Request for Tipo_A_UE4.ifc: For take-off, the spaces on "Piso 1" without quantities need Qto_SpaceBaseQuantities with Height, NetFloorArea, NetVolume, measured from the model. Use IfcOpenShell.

First a look at what the model holds.

```python
import ifcopenshell
import ifcopenshell.util.element
import ifcopenshell.util.unit

model = ifcopenshell.open("Tipo_A_UE4.ifc")
print(model.schema)
for unit_type in ("LENGTHUNIT", "AREAUNIT", "VOLUMEUNIT"):
    print(unit_type, ifcopenshell.util.unit.calculate_unit_scale(model, unit_type))
storey = next(s for s in model.by_type("IfcBuildingStorey") if s.Name == "Piso 1")
spaces = [e for e in ifcopenshell.util.element.get_decomposition(storey) if e.is_a("IfcSpace")]
for e in sorted(spaces, key=lambda e: e.id()):
    print(e.id(), e.is_a(), e.Name, list(ifcopenshell.util.element.get_psets(e, qtos_only=True)), sep=" | ")
```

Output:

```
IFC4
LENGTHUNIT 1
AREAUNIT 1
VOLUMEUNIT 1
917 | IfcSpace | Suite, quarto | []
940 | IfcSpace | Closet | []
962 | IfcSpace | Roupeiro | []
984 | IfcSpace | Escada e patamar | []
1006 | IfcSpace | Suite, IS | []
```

```python
import ifcopenshell
import ifcopenshell.api.pset
import ifcopenshell.geom
import ifcopenshell.util.element
import ifcopenshell.util.shape
import ifcopenshell.util.unit

model = ifcopenshell.open("Tipo_A_UE4.ifc")
unit_scale = ifcopenshell.util.unit.calculate_unit_scale(model)
area_scale = ifcopenshell.util.unit.calculate_unit_scale(model, "AREAUNIT")
volume_scale = ifcopenshell.util.unit.calculate_unit_scale(model, "VOLUMEUNIT")
settings = ifcopenshell.geom.settings()

storey = next(s for s in model.by_type("IfcBuildingStorey") if s.Name == "Piso 1")
spaces = [e for e in ifcopenshell.util.element.get_decomposition(storey) if e.is_a("IfcSpace")]

for e in sorted(spaces, key=lambda e: e.id()):
    if ifcopenshell.util.element.get_psets(e, qtos_only=True, should_inherit=False):
        continue
    # Geometry comes back in metres, in the element's own axes.
    shape = ifcopenshell.geom.create_shape(settings, e)
    values = {
        "Height": ifcopenshell.util.shape.get_z(shape.geometry) / unit_scale,
        "NetFloorArea": ifcopenshell.util.shape.get_footprint_area(shape.geometry) / area_scale,
        "NetVolume": ifcopenshell.util.shape.get_volume(shape.geometry) / volume_scale,
    }
    qto = ifcopenshell.api.pset.add_qto(model, product=e, name="Qto_SpaceBaseQuantities")
    ifcopenshell.api.pset.edit_qto(model, qto=qto, properties=values)
    print(e.id(), {k: round(v, 3) for k, v in values.items()})

model.write("Tipo_A_UE4-out.ifc")
```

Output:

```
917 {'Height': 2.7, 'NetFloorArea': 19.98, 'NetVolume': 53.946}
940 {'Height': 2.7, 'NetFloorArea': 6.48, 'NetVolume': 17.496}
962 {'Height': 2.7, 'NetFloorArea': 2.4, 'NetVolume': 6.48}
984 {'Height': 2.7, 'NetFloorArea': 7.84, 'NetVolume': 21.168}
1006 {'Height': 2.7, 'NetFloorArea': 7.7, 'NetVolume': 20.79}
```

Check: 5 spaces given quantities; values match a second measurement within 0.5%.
